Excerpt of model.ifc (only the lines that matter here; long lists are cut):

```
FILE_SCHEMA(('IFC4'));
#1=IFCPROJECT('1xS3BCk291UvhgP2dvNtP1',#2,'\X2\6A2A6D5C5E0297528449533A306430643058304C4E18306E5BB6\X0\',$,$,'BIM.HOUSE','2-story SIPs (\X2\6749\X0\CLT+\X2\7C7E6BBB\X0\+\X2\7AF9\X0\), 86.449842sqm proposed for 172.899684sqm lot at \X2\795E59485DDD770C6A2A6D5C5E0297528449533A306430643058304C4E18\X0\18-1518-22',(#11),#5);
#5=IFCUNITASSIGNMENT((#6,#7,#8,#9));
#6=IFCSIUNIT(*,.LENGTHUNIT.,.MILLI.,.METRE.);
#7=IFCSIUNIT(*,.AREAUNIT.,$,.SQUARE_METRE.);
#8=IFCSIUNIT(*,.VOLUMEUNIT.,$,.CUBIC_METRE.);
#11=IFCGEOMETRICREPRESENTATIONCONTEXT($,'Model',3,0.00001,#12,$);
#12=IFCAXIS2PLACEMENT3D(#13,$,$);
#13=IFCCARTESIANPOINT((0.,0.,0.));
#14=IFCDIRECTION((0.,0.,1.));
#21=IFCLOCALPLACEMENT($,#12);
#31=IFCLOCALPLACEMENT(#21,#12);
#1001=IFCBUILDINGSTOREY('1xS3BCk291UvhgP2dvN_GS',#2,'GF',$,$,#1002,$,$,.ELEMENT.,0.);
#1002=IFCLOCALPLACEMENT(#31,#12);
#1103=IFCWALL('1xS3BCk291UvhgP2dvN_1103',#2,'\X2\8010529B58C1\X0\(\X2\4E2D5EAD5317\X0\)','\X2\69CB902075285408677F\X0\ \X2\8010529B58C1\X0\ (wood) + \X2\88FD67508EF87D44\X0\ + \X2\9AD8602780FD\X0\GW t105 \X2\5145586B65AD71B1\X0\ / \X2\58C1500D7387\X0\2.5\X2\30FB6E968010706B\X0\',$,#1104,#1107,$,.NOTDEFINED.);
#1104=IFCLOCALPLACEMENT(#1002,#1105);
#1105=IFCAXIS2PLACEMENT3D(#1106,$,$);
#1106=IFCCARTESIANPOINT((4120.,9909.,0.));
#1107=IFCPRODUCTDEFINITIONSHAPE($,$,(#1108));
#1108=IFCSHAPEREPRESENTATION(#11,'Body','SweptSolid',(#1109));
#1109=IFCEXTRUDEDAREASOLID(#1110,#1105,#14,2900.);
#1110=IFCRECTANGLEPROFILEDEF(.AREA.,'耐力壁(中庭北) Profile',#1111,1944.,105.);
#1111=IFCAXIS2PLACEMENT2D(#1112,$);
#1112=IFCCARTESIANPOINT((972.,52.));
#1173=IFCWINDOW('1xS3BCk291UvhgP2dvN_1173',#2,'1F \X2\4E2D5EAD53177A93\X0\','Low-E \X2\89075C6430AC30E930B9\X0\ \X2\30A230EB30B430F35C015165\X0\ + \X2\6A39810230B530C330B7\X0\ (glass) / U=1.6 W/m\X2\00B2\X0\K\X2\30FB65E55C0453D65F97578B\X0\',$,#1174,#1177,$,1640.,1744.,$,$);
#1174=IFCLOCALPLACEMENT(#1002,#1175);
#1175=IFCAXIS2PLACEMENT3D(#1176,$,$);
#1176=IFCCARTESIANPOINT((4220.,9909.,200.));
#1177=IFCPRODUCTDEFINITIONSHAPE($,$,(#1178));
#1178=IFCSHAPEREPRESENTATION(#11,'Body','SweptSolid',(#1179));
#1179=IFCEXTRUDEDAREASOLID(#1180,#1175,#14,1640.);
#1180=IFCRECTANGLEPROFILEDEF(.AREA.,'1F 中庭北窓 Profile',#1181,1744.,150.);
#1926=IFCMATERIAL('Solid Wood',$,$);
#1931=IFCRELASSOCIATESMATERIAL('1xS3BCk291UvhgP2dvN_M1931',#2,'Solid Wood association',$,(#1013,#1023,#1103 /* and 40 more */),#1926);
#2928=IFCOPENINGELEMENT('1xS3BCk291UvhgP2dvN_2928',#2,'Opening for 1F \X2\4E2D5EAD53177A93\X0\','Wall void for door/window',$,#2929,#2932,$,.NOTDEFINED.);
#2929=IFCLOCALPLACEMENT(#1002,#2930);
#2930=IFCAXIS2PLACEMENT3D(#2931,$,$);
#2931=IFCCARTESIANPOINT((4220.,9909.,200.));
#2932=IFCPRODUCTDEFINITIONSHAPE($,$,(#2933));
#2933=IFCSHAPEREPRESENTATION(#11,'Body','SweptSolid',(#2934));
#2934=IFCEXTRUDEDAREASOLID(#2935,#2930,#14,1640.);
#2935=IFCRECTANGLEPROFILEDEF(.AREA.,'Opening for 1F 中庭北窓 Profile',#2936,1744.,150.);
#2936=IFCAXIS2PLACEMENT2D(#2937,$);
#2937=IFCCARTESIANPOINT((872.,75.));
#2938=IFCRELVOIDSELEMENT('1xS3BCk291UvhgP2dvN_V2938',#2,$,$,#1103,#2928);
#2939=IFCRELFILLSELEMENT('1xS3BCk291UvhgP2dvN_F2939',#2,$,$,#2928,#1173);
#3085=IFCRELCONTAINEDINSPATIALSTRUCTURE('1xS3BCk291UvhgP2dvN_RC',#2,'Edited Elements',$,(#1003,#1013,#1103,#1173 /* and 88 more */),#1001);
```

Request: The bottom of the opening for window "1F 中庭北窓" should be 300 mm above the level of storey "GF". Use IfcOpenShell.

```python
import numpy as np
import ifcopenshell
import ifcopenshell.api.geometry
import ifcopenshell.geom
import ifcopenshell.util.element
import ifcopenshell.util.placement
import ifcopenshell.util.shape
import ifcopenshell.util.unit

model = ifcopenshell.open("model.ifc")
unit_scale = ifcopenshell.util.unit.calculate_unit_scale(model)

window = model.by_guid("1xS3BCk291UvhgP2dvN_1173")
opening = window.FillsVoids[0].RelatingOpeningElement
storey = ifcopenshell.util.element.get_container(window, ifc_class="IfcBuildingStorey")
level = ifcopenshell.util.placement.get_local_placement(storey.ObjectPlacement)[2, 3]

# The opening's origin need not be at the sill, so measure its lowest point.
shape = ifcopenshell.geom.create_shape(ifcopenshell.geom.settings(), opening)
bottom = ifcopenshell.util.shape.get_shape_bottom_elevation(shape, shape.geometry) / unit_scale
dz = level + 300.0 - bottom

shift = np.array([0.0, 0.0, dz])
# The window is not placed relative to its opening, so move both.
for product in (opening, window):
    matrix = ifcopenshell.util.placement.get_local_placement(product.ObjectPlacement)
    matrix[:3, 3] += shift
    ifcopenshell.api.geometry.edit_object_placement(model, product=product, matrix=matrix, is_si=False)

print(f"moved by {dz * unit_scale:+.3f} m")

model.write("model_edited.ifc")
```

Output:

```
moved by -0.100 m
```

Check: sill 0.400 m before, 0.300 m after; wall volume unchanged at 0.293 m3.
